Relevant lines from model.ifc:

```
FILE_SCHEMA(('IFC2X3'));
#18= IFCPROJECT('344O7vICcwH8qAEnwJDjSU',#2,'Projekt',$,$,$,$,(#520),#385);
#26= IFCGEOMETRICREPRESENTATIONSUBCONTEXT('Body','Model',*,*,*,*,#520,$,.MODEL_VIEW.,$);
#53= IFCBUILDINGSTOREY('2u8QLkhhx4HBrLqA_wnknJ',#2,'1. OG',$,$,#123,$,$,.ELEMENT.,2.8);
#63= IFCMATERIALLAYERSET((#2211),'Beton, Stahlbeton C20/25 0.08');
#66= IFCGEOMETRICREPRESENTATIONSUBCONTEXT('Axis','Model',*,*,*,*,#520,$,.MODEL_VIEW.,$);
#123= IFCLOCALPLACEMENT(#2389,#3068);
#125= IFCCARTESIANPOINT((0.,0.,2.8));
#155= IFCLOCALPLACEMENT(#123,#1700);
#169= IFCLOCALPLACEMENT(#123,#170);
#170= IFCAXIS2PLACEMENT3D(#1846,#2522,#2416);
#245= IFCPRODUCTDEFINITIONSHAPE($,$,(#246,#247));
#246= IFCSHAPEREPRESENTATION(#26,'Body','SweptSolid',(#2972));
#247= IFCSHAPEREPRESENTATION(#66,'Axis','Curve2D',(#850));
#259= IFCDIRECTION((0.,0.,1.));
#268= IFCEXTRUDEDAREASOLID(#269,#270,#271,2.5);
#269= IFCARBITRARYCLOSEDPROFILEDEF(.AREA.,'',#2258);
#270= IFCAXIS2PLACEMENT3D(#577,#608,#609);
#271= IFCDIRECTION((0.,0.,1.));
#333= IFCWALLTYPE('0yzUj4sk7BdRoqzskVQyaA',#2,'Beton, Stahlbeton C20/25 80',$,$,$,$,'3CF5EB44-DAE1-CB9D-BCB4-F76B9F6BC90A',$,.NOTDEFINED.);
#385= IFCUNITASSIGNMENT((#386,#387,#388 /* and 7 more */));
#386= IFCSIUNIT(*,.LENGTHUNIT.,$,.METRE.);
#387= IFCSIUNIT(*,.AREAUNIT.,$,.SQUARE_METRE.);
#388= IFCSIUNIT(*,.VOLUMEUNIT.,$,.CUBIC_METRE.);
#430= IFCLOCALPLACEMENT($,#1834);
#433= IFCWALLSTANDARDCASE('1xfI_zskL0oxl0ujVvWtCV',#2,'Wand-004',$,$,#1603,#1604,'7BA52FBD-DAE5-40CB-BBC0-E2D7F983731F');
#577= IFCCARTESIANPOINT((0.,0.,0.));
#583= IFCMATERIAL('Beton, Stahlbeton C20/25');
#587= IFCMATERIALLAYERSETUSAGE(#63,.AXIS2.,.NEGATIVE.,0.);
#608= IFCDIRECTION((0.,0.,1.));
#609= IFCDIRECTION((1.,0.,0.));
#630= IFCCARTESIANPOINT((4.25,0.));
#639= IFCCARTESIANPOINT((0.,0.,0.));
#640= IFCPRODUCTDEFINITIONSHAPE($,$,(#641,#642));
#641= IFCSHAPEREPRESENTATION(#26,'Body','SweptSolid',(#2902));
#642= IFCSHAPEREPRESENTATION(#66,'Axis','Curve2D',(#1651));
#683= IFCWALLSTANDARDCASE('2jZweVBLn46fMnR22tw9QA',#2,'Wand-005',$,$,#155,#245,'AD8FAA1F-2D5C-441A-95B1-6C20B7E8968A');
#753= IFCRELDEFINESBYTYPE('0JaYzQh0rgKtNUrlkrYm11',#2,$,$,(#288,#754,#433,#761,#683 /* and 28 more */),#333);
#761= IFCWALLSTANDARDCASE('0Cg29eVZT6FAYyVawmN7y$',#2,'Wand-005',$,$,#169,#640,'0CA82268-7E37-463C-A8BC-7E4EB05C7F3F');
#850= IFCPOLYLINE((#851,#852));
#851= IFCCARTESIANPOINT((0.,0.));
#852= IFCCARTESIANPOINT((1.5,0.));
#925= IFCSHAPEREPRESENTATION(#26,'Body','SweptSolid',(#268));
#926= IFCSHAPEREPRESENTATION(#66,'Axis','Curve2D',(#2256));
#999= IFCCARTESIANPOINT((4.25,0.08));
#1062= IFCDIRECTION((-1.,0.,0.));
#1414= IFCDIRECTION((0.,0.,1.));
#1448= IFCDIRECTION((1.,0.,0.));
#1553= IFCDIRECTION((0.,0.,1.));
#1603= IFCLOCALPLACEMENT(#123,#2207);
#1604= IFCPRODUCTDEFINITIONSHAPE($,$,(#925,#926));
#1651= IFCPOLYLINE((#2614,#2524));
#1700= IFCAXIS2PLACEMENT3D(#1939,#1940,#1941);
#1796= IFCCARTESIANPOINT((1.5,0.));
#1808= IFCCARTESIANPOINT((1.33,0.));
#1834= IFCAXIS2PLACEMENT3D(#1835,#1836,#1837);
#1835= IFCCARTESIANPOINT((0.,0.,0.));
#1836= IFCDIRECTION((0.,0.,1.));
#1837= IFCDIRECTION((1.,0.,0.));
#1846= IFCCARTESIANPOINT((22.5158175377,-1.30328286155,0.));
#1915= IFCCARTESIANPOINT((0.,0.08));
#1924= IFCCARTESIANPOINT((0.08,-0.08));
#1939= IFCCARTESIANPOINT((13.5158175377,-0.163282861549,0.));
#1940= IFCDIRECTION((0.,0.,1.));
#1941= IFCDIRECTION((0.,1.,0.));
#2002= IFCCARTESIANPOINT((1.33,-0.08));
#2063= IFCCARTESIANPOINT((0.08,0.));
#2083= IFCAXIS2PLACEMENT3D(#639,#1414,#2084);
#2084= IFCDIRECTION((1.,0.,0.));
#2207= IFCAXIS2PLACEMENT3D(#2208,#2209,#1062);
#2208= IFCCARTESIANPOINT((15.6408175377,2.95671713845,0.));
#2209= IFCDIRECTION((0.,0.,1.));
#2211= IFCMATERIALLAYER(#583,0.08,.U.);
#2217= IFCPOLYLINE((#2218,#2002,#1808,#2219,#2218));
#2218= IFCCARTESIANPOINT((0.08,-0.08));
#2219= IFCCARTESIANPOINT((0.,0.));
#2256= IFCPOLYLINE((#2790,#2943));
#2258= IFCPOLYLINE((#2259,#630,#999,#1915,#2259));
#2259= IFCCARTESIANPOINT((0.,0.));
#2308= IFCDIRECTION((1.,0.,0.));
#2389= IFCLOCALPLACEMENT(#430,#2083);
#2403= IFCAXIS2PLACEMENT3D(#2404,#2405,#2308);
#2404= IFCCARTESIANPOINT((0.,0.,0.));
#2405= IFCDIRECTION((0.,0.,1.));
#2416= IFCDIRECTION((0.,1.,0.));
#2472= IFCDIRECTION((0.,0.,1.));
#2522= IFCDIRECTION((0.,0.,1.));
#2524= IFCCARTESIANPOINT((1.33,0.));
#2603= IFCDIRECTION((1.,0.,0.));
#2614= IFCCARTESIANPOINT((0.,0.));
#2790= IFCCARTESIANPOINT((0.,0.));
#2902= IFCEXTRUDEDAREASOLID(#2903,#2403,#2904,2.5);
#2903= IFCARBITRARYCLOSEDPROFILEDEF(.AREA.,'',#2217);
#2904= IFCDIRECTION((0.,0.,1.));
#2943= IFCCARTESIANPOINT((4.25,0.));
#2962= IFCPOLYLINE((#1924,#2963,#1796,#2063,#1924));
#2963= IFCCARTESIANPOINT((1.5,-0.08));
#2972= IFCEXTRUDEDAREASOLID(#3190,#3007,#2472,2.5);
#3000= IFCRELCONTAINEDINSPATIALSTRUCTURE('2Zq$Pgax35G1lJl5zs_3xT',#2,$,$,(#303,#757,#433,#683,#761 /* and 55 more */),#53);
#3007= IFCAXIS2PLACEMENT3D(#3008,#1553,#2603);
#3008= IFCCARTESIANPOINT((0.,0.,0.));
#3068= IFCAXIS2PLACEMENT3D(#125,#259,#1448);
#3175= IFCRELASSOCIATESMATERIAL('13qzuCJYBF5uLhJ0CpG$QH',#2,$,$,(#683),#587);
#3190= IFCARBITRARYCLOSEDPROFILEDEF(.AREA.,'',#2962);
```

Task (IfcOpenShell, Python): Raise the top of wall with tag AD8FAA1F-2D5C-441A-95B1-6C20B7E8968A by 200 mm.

```python
import ifcopenshell
import ifcopenshell.geom
import ifcopenshell.util.representation
import ifcopenshell.util.shape

model = ifcopenshell.open("model.ifc")
settings = ifcopenshell.geom.settings()


def volume(element):
    """Net volume in cubic metres, openings subtracted."""
    shape = ifcopenshell.geom.create_shape(settings, element)
    return ifcopenshell.util.shape.get_volume(shape.geometry)


wall = model.by_guid("2jZweVBLn46fMnR22tw9QA")
before = volume(wall)

body = ifcopenshell.util.representation.get_representation(wall, "Model", "Body")
solid = body.Items[0]
old_height = solid.Depth
solid.Depth += 0.2
after = volume(wall)

print(f"height {old_height:g} -> {solid.Depth:g}, volume {before:.3f} -> {after:.3f} m3")

model.write("model_updated.ifc")
```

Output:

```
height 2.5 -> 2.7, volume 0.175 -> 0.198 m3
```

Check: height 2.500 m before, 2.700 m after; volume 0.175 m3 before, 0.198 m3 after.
